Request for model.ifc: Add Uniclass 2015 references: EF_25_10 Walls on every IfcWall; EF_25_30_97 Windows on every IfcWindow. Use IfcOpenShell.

First a look at what the model holds.

```python
import ifcopenshell

model = ifcopenshell.open("model.ifc")
print(model.schema)
print("classifications:", [c.Name for c in model.by_type("IfcClassification")])
for ifc_class in ("IfcDoor", "IfcRoof", "IfcStair", "IfcWall", "IfcWindow"):
    print(ifc_class, len(model.by_type(ifc_class)))
```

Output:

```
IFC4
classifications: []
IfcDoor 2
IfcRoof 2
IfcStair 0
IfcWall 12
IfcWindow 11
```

```python
import ifcopenshell
import ifcopenshell.api.classification

model = ifcopenshell.open("model.ifc")

system = ifcopenshell.api.classification.add_classification(model, classification="Uniclass 2015")

codes = {
    "IfcWall": ("EF_25_10", "Walls"),
    "IfcWindow": ("EF_25_30_97", "Windows"),
}
for ifc_class, (code, name) in codes.items():
    products = model.by_type(ifc_class)
    ifcopenshell.api.classification.add_reference(
        model, products=products, classification=system, identification=code, name=name
    )
    print(code, len(products))

model.write("model-out.ifc")
```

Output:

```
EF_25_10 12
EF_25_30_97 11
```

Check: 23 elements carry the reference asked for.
